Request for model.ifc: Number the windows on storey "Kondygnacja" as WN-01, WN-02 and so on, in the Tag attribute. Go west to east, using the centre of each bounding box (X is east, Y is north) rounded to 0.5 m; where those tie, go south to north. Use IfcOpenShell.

First a look at what the model holds.

```python
import ifcopenshell
import ifcopenshell.util.element
import ifcopenshell.util.placement

model = ifcopenshell.open("model.ifc")
print(model.schema)
storey = next(s for s in model.by_type("IfcBuildingStorey") if s.Name == "Kondygnacja")
windows = [e for e in ifcopenshell.util.element.get_decomposition(storey) if e.is_a("IfcWindow")]
for e in sorted(windows, key=lambda e: e.id()):
    origin = ifcopenshell.util.placement.get_local_placement(e.ObjectPlacement)[:3, 3]
    print(e.id(), e.Tag, e.Name, origin.round(2) + 0.0, sep=" | ")
```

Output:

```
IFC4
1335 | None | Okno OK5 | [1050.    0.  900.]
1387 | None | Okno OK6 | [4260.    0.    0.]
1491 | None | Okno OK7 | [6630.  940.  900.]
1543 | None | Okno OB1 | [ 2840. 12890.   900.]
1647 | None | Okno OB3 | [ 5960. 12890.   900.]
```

```python
import ifcopenshell
import ifcopenshell.geom
import ifcopenshell.util.element
import ifcopenshell.util.shape

model = ifcopenshell.open("model.ifc")
settings = ifcopenshell.geom.settings()
settings.set("use-world-coords", True)


def centre(element):
    shape = ifcopenshell.geom.create_shape(settings, element)
    return ifcopenshell.util.shape.get_bbox_centroid(shape.geometry)


storey = next(s for s in model.by_type("IfcBuildingStorey") if s.Name == "Kondygnacja")
windows = [e for e in ifcopenshell.util.element.get_decomposition(storey) if e.is_a("IfcWindow")]

# Insertion points can sit at a corner or the storey origin, so sort by the geometry (in metres).
centres = {e: centre(e) for e in windows}
windows.sort(key=lambda e: (round(centres[e][0] / 0.5), centres[e][1]))

for i, e in enumerate(windows, start=1):
    number = f"WN-{i:02d}"
    e.Tag = number
    print(e.id(), number)

model.write("model_rev.ifc")
```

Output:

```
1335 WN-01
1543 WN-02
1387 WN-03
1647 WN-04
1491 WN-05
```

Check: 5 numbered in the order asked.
